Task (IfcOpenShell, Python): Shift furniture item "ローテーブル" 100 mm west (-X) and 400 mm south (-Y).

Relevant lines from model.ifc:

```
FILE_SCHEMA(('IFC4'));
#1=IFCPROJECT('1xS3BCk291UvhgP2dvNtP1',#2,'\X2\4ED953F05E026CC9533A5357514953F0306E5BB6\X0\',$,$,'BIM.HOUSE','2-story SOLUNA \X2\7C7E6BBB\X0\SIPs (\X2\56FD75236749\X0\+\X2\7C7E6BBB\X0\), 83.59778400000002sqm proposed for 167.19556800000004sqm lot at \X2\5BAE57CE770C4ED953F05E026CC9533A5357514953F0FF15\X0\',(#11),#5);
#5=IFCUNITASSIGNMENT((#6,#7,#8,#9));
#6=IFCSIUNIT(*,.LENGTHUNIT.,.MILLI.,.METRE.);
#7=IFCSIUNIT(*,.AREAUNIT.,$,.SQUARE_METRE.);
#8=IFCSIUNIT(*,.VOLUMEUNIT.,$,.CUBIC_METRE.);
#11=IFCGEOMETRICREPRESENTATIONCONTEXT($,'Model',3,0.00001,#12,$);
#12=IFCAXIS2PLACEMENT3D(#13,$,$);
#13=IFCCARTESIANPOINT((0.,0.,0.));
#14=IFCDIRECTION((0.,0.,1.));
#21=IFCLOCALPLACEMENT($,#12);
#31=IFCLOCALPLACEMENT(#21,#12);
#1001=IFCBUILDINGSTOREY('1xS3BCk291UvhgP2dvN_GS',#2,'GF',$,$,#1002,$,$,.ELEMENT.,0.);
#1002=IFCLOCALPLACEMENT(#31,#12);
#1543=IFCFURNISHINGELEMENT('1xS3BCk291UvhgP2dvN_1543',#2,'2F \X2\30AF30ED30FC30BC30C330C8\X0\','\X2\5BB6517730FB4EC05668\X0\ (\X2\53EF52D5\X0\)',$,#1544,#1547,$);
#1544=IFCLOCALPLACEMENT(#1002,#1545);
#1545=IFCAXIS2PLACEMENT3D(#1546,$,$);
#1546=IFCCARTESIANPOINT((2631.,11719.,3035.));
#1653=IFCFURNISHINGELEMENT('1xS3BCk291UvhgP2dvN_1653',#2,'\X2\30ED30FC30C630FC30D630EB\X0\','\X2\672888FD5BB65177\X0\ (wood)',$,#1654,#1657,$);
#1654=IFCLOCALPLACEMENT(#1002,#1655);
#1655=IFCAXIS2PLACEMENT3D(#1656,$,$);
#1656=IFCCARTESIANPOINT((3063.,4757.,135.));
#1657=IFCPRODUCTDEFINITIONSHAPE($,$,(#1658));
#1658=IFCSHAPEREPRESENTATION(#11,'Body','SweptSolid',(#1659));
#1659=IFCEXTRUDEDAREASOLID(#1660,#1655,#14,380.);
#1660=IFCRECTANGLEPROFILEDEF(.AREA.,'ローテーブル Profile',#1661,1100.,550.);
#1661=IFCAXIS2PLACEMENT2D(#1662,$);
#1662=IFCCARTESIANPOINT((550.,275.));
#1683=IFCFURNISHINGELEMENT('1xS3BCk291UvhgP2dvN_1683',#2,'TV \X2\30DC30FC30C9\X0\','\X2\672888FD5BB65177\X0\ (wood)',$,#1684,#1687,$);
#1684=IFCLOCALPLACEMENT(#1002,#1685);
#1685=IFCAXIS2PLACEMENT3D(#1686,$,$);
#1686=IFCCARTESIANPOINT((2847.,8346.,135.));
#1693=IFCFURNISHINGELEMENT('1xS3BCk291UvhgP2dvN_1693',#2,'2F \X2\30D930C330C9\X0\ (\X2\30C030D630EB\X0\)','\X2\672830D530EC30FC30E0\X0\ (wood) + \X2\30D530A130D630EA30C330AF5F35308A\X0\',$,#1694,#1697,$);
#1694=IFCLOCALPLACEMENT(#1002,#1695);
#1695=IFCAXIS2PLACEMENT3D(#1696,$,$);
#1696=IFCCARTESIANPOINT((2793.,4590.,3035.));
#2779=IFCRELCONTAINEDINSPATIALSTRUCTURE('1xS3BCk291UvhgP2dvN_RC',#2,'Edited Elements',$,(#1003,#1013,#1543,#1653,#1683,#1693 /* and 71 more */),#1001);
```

```python
import ifcopenshell
import ifcopenshell.api.geometry
import ifcopenshell.util.placement
import ifcopenshell.util.unit

model = ifcopenshell.open("model.ifc")
unit_scale = ifcopenshell.util.unit.calculate_unit_scale(model)

item = model.by_id(1653)
matrix = ifcopenshell.util.placement.get_local_placement(item.ObjectPlacement)
matrix[0, 3] -= 0.1 / unit_scale
matrix[1, 3] -= 0.4 / unit_scale
ifcopenshell.api.geometry.edit_object_placement(model, product=item, matrix=matrix, is_si=False)

print(ifcopenshell.util.placement.get_local_placement(item.ObjectPlacement).round(3) + 0.0)

model.write("model_v2.ifc")
```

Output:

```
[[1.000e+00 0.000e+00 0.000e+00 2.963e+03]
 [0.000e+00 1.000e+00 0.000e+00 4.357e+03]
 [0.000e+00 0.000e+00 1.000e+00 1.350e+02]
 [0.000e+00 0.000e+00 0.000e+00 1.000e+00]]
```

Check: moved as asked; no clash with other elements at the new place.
